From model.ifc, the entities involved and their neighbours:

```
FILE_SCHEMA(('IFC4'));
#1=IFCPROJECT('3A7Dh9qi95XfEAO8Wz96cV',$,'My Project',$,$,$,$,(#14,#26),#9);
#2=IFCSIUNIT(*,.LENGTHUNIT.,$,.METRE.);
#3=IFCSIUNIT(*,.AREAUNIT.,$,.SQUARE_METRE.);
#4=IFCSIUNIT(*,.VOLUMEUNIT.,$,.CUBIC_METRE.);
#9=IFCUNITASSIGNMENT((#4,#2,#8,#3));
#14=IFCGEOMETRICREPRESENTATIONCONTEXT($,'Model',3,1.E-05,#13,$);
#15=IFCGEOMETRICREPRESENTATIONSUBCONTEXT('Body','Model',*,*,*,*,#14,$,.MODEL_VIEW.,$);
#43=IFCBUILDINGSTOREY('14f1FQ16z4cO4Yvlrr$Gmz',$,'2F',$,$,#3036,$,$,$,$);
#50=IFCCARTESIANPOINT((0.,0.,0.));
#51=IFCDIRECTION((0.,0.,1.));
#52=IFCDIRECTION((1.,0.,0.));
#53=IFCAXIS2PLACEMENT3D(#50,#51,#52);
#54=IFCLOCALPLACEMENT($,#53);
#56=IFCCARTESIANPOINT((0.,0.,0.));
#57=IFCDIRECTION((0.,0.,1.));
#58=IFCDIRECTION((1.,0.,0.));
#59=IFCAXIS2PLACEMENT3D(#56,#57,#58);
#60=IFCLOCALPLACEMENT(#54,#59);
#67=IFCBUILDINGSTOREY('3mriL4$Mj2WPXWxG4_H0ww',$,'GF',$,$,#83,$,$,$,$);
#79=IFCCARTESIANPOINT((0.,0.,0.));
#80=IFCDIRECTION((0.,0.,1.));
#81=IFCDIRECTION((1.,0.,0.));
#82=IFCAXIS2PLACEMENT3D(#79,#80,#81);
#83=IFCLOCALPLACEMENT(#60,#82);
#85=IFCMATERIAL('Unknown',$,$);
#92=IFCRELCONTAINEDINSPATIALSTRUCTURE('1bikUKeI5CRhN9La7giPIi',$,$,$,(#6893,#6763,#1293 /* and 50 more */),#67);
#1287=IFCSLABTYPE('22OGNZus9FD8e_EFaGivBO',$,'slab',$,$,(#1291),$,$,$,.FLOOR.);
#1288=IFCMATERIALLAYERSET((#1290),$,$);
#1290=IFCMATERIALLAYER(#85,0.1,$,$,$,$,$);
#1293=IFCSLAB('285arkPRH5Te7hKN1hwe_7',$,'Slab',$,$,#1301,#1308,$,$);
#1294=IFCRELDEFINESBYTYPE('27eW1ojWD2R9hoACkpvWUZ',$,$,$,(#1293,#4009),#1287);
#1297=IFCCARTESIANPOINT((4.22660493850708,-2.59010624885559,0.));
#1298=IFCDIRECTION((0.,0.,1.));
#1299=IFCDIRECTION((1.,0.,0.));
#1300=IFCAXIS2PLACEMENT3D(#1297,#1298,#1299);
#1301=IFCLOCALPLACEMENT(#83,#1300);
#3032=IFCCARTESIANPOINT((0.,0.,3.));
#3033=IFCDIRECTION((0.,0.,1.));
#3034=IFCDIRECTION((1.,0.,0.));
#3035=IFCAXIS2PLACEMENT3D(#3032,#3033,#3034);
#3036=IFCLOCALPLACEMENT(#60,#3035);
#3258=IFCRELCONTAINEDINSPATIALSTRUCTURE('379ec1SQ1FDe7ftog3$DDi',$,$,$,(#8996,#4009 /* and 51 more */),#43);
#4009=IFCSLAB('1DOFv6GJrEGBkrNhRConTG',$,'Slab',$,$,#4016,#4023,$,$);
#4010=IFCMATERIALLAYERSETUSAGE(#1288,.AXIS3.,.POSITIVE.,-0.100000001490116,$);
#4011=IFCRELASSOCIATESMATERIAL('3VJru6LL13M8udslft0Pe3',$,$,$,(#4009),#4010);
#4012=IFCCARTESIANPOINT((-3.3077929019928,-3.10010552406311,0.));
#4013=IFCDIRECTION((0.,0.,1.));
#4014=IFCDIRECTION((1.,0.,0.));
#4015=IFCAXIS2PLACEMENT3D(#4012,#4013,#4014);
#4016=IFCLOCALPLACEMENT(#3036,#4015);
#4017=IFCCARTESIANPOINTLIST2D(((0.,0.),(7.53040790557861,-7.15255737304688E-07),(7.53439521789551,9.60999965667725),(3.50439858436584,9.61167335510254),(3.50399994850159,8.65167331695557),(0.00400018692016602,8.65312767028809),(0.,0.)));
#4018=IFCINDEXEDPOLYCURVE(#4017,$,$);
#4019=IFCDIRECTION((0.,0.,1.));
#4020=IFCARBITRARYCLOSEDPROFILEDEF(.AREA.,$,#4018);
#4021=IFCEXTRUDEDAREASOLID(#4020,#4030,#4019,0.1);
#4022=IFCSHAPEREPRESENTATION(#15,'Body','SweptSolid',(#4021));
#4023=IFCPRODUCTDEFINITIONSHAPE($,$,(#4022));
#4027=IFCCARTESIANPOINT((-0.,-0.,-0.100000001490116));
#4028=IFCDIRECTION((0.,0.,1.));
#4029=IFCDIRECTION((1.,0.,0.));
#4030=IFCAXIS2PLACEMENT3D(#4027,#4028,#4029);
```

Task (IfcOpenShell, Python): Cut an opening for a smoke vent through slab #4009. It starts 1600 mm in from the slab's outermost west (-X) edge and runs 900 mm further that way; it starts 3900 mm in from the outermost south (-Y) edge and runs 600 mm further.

```python
import numpy as np
import ifcopenshell
import ifcopenshell.api.feature
import ifcopenshell.api.geometry
import ifcopenshell.api.root
import ifcopenshell.geom
import ifcopenshell.util.placement
import ifcopenshell.util.representation
import ifcopenshell.util.shape
import ifcopenshell.util.unit

model = ifcopenshell.open("model.ifc")
unit_scale = ifcopenshell.util.unit.calculate_unit_scale(model)
settings = ifcopenshell.geom.settings()


def volume(element):
    """Net volume in cubic metres, openings subtracted."""
    shape = ifcopenshell.geom.create_shape(settings, element)
    return ifcopenshell.util.shape.get_volume(shape.geometry)


slab = model.by_guid("1DOFv6GJrEGBkrNhRConTG")
before = volume(slab)

# Extent in the slab's own axes, in metres. The edges named are its -X and -Y sides.
slab_shape = ifcopenshell.geom.create_shape(settings, slab)
vertices = ifcopenshell.util.shape.get_vertices(slab_shape.geometry)
x_min, y_min, bottom = vertices.min(axis=0)
top = vertices[:, 2].max()

opening = ifcopenshell.api.root.create_entity(model, ifc_class="IfcOpeningElement", name="Smoke vent opening", predefined_type="OPENING")
context = ifcopenshell.util.representation.get_context(model, "Model", "Body", "MODEL_VIEW")
width, depth = 0.9, 0.6
outline = [(0.0, 0.0), (width, 0.0), (width, depth), (0.0, depth), (0.0, 0.0)]
# Overshoot both faces by 50 mm so the cut is clean.
shape = ifcopenshell.api.geometry.add_slab_representation(
    model, context=context, depth=top - bottom + 0.1, polyline=outline
)
ifcopenshell.api.geometry.assign_representation(model, product=opening, representation=shape)

matrix = ifcopenshell.util.placement.get_local_placement(slab.ObjectPlacement)
matrix[:, 3] = matrix @ np.append(np.array([x_min + 1.6, y_min + 3.9, bottom - 0.05]) / unit_scale, 1.0)
ifcopenshell.api.geometry.edit_object_placement(model, product=opening, matrix=matrix, is_si=False)
ifcopenshell.api.feature.add_feature(model, feature=opening, element=slab)

after = volume(slab)

print(f"slab volume {before:.3f} -> {after:.3f} m3")

model.write("model_rev.ifc")
```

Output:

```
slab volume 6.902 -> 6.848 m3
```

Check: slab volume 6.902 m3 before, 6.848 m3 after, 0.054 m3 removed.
